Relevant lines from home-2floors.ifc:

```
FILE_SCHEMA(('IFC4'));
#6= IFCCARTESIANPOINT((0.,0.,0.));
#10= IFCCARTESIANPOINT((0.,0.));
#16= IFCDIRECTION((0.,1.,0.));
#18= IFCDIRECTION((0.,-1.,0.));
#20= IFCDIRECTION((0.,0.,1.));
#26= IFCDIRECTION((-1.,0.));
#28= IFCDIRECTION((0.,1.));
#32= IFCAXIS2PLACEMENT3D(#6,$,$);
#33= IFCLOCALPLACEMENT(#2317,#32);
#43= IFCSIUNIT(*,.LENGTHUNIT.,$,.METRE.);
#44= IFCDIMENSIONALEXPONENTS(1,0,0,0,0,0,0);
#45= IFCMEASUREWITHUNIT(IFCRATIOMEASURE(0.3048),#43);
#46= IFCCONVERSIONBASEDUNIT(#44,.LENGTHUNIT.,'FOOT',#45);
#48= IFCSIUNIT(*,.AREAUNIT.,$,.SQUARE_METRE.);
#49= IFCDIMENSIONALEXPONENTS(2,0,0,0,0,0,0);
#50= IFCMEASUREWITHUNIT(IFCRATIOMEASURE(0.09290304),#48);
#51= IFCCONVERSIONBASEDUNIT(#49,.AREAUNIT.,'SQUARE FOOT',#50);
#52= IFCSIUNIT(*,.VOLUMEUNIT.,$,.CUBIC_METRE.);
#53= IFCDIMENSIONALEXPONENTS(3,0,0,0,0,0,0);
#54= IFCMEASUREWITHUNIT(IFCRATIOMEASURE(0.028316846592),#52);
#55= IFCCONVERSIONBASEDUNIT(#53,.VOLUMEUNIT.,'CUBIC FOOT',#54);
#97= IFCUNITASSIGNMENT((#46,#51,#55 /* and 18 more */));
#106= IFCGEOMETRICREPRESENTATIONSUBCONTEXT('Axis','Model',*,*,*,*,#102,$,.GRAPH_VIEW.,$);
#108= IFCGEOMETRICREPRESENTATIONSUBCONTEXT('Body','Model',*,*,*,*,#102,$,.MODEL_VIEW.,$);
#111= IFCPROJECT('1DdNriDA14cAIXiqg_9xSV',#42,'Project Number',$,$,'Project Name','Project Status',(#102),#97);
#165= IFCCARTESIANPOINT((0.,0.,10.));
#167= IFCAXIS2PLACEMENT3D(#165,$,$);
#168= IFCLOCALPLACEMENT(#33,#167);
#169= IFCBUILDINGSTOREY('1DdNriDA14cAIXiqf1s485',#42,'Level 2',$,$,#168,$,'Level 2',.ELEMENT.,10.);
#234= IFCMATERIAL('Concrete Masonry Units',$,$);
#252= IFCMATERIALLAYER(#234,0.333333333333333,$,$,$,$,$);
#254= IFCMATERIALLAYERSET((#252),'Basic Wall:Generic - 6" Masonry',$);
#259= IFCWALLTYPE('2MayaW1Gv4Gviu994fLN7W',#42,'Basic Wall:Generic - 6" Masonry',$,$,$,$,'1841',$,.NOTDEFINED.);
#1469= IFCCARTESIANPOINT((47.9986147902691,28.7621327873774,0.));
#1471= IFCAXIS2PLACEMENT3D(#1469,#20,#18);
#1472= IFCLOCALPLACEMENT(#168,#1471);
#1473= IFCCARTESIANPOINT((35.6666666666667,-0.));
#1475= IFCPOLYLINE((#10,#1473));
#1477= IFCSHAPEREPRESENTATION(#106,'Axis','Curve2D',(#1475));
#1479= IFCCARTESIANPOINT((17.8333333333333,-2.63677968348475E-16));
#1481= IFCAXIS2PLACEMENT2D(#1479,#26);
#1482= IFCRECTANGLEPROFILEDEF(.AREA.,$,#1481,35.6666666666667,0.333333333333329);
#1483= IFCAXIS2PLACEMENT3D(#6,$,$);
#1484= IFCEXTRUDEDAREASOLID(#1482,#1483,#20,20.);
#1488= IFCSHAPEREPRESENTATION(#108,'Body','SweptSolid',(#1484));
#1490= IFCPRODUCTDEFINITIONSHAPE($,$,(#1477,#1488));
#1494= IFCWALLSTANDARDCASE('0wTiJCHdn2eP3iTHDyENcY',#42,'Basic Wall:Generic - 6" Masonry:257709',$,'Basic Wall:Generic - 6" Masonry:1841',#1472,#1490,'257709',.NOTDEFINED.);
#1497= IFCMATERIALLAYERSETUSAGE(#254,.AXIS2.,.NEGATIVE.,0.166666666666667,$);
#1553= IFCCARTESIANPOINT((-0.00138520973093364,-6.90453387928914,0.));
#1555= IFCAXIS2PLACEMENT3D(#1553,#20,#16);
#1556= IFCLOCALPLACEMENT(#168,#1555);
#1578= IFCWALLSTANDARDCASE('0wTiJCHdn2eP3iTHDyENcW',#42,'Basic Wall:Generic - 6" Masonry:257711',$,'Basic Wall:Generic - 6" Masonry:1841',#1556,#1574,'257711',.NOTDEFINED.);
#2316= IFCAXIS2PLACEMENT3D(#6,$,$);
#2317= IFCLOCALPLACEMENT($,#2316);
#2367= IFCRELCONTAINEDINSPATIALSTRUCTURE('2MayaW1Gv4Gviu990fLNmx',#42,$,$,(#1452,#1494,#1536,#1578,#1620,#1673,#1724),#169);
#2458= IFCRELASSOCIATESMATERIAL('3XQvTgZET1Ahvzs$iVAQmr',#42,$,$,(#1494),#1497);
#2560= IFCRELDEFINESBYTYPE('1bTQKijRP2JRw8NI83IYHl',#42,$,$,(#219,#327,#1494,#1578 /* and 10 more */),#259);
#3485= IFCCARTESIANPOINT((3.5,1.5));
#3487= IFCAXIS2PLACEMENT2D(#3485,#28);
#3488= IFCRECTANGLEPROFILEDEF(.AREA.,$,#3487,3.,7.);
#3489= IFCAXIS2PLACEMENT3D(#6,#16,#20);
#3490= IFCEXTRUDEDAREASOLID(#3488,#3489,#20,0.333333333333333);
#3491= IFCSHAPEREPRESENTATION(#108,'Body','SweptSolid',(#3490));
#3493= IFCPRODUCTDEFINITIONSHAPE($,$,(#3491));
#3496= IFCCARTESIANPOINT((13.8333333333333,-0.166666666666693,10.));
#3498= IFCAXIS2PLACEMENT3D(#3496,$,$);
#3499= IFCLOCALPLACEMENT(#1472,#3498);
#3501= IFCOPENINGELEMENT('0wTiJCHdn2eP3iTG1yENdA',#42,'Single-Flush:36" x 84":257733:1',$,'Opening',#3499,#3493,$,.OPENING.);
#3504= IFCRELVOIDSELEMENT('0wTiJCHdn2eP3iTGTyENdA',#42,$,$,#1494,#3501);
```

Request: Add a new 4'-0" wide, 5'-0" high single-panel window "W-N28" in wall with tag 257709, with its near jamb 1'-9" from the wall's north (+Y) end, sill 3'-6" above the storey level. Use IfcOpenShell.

```python
import numpy as np
import ifcopenshell
import ifcopenshell.api.feature
import ifcopenshell.api.geometry
import ifcopenshell.api.root
import ifcopenshell.api.spatial
import ifcopenshell.geom
import ifcopenshell.util.element
import ifcopenshell.util.placement
import ifcopenshell.util.representation
import ifcopenshell.util.shape
import ifcopenshell.util.unit

model = ifcopenshell.open("home-2floors.ifc")
unit_scale = ifcopenshell.util.unit.calculate_unit_scale(model)
settings = ifcopenshell.geom.settings()


def volume(element):
    """Net volume in cubic metres, openings subtracted."""
    shape = ifcopenshell.geom.create_shape(settings, element)
    return ifcopenshell.util.shape.get_volume(shape.geometry)


wall = model.by_guid("0wTiJCHdn2eP3iTHDyENcY")
storey = ifcopenshell.util.element.get_container(wall, ifc_class="IfcBuildingStorey")
context = ifcopenshell.util.representation.get_context(model, "Model", "Body", "MODEL_VIEW")
before = volume(wall)

width, height, from_end, sill = 1.2192, 1.524, 0.5334, 1.0668  # metres

# The wall runs along its own X axis, and the end named is its -X end.
wall_shape = ifcopenshell.geom.create_shape(settings, wall)
x, y, z = ifcopenshell.util.shape.get_vertices(wall_shape.geometry).T
start = x.min() + from_end
face, thickness = float(y.min()), float(y.max() - y.min())
wall_matrix = ifcopenshell.util.placement.get_local_placement(wall.ObjectPlacement)
level = ifcopenshell.util.placement.get_local_placement(storey.ObjectPlacement)[2, 3]


def in_wall(x, y):
    """Placement at x, y metres in the wall's axes, at sill height."""
    matrix = wall_matrix.copy()
    matrix[:, 3] = wall_matrix @ np.array([x / unit_scale, y / unit_scale, 0.0, 1.0])
    matrix[2, 3] = level + sill / unit_scale
    return matrix


# Opening: a box that overshoots both wall faces by 50 mm.
opening = ifcopenshell.api.root.create_entity(model, ifc_class="IfcOpeningElement", predefined_type="OPENING")
box = ifcopenshell.api.geometry.add_wall_representation(
    model, context=context, length=width, height=height, thickness=thickness + 0.1
)
ifcopenshell.api.geometry.assign_representation(model, product=opening, representation=box)
ifcopenshell.api.geometry.edit_object_placement(model, product=opening, matrix=in_wall(start, face - 0.05), is_si=False)
ifcopenshell.api.feature.add_feature(model, feature=opening, element=wall)

window = ifcopenshell.api.root.create_entity(model, ifc_class="IfcWindow", name="W-N28", predefined_type="WINDOW")
window.OverallWidth, window.OverallHeight = width / unit_scale, height / unit_scale
window.PartitioningType = "SINGLE_PANEL"
body = ifcopenshell.api.geometry.add_window_representation(
    model,
    context=context,
    overall_width=window.OverallWidth,
    overall_height=window.OverallHeight,
    partition_type="SINGLE_PANEL",
)
ifcopenshell.api.geometry.assign_representation(model, product=window, representation=body)
ifcopenshell.api.spatial.assign_container(model, products=[window], relating_structure=storey)
ifcopenshell.api.feature.add_filling(model, opening=opening, element=window)

# Centre the window in the wall's thickness.
ifcopenshell.api.geometry.edit_object_placement(model, product=window, matrix=in_wall(start, face), is_si=False)
window_shape = ifcopenshell.geom.create_shape(settings, window)
depth = ifcopenshell.util.shape.get_vertices(window_shape.geometry)[:, 1]
offset = face + thickness / 2 - (depth.min() + depth.max()) / 2
ifcopenshell.api.geometry.edit_object_placement(model, product=window, matrix=in_wall(start, offset), is_si=False)

after = volume(wall)

print(f"wall volume {before:.3f} -> {after:.3f} m3")

model.write("home-2floors_updated.ifc")
```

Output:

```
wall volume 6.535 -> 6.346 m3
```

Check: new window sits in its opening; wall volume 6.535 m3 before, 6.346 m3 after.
